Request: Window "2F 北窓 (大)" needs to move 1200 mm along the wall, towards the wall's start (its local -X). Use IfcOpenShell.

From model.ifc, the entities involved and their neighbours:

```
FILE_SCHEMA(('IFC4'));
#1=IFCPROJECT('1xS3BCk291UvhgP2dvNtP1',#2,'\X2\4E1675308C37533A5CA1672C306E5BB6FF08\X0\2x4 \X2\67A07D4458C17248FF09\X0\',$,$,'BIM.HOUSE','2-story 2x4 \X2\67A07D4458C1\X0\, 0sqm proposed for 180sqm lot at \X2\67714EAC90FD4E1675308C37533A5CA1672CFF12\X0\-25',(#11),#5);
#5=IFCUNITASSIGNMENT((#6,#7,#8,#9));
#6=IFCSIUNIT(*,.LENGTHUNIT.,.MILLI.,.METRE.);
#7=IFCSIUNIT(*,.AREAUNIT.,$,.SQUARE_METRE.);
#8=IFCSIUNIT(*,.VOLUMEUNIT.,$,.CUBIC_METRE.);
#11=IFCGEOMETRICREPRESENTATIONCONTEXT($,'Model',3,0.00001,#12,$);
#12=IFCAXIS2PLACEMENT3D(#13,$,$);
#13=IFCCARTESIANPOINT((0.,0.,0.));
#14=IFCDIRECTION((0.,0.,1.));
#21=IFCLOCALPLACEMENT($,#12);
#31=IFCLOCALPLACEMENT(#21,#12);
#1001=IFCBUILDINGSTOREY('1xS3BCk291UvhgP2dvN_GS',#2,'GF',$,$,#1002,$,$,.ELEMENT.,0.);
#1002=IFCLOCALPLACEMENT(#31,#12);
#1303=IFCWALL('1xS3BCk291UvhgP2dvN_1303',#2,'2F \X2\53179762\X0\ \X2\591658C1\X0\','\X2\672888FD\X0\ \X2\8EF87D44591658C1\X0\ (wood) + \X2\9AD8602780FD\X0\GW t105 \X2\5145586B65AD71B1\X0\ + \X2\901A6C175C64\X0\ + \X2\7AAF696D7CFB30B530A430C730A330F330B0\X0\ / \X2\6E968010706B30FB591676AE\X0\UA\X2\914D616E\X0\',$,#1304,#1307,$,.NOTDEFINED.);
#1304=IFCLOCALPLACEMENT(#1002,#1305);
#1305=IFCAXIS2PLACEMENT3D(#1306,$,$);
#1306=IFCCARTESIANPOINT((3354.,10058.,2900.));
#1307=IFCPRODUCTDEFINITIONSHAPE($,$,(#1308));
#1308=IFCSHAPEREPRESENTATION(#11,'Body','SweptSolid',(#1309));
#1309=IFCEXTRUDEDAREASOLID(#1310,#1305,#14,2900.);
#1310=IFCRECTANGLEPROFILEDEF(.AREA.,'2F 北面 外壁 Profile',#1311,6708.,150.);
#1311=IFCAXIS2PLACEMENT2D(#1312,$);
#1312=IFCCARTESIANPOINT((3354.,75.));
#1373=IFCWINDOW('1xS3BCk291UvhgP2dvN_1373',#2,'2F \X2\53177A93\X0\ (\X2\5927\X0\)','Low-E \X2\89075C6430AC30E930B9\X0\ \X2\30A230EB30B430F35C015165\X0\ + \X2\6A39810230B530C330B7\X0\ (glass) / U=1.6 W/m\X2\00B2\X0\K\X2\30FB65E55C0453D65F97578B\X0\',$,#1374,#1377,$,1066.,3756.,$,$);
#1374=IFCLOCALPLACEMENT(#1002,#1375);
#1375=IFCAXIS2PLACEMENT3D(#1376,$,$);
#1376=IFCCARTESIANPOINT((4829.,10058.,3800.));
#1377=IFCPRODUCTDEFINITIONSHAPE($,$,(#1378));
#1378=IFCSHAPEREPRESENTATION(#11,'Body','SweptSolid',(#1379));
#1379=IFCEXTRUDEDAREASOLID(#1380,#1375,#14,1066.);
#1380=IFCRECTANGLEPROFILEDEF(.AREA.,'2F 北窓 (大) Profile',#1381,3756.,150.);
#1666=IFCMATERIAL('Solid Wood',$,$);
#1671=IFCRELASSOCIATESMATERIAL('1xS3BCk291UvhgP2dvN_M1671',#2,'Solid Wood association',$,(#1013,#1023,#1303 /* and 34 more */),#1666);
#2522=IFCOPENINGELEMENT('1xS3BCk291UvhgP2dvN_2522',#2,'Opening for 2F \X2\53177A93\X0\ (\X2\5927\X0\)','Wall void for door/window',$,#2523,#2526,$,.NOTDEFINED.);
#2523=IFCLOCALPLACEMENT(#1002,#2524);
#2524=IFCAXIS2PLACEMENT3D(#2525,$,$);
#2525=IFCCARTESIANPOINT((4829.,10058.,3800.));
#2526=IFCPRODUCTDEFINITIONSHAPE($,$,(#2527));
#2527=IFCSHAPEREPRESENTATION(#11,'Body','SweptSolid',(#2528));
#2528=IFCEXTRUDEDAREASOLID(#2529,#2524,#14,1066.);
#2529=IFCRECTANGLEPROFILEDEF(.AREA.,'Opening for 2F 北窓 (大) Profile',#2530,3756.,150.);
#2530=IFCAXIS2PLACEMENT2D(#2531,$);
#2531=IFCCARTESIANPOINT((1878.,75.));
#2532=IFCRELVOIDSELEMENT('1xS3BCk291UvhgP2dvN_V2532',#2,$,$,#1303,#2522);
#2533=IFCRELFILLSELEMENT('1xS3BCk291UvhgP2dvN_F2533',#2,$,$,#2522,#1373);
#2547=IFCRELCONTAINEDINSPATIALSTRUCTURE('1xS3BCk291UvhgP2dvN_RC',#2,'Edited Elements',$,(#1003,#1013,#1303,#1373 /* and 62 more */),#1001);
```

```python
import ifcopenshell
import ifcopenshell.api.geometry
import ifcopenshell.util.placement

model = ifcopenshell.open("model.ifc")

window = model.by_guid("1xS3BCk291UvhgP2dvN_1373")
opening = window.FillsVoids[0].RelatingOpeningElement
wall = opening.VoidsElements[0].RelatingBuildingElement

wall_matrix = ifcopenshell.util.placement.get_local_placement(wall.ObjectPlacement)
shift = wall_matrix[:3, 0] * -1200.0
before = ifcopenshell.util.placement.get_local_placement(window.ObjectPlacement)[:3, 3].copy()

# The window is not placed relative to its opening, so move both.
for product in (opening, window):
    matrix = ifcopenshell.util.placement.get_local_placement(product.ObjectPlacement)
    matrix[:3, 3] += shift
    ifcopenshell.api.geometry.edit_object_placement(model, product=product, matrix=matrix, is_si=False)

after = ifcopenshell.util.placement.get_local_placement(window.ObjectPlacement)[:3, 3]
print("window moved by", (after - before).round(3) + 0.0)

model.write("model_edited.ifc")
```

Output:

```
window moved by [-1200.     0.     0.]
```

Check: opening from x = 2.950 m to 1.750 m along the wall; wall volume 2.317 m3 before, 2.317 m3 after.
